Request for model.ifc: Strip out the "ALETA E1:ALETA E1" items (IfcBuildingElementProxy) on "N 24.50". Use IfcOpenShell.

First a look at what the model holds.

```python
import ifcopenshell
import ifcopenshell.util.element

model = ifcopenshell.open("model.ifc")
print(model.schema)
storey = next(s for s in model.by_type("IfcBuildingStorey") if s.Name == "N 24.50")
proxies = [e for e in ifcopenshell.util.element.get_decomposition(storey) if e.is_a("IfcBuildingElementProxy")]
seen = {}
for e in proxies:
    element_type = ifcopenshell.util.element.get_type(e)
    name = element_type.Name if element_type not in (None, e) else None
    seen[name] = seen.get(name, 0) + 1
for name, count in sorted(seen.items(), key=str):
    print(count, "x", name)
```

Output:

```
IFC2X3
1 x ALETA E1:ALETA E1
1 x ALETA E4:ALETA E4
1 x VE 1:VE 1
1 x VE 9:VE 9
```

```python
import ifcopenshell
import ifcopenshell.api.root
import ifcopenshell.util.element

model = ifcopenshell.open("model.ifc")

storey = next(s for s in model.by_type("IfcBuildingStorey") if s.Name == "N 24.50")
proxies = [e for e in ifcopenshell.util.element.get_decomposition(storey) if e.is_a("IfcBuildingElementProxy")]
targets = [e for e in proxies if (t := ifcopenshell.util.element.get_type(e)) not in (None, e) and t.Name == "ALETA E1:ALETA E1"]

for e in targets:
    ifcopenshell.api.root.remove_product(model, product=e)
print(len(targets), "removed")

model.write("model_edited.ifc")
```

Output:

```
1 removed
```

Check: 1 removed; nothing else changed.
